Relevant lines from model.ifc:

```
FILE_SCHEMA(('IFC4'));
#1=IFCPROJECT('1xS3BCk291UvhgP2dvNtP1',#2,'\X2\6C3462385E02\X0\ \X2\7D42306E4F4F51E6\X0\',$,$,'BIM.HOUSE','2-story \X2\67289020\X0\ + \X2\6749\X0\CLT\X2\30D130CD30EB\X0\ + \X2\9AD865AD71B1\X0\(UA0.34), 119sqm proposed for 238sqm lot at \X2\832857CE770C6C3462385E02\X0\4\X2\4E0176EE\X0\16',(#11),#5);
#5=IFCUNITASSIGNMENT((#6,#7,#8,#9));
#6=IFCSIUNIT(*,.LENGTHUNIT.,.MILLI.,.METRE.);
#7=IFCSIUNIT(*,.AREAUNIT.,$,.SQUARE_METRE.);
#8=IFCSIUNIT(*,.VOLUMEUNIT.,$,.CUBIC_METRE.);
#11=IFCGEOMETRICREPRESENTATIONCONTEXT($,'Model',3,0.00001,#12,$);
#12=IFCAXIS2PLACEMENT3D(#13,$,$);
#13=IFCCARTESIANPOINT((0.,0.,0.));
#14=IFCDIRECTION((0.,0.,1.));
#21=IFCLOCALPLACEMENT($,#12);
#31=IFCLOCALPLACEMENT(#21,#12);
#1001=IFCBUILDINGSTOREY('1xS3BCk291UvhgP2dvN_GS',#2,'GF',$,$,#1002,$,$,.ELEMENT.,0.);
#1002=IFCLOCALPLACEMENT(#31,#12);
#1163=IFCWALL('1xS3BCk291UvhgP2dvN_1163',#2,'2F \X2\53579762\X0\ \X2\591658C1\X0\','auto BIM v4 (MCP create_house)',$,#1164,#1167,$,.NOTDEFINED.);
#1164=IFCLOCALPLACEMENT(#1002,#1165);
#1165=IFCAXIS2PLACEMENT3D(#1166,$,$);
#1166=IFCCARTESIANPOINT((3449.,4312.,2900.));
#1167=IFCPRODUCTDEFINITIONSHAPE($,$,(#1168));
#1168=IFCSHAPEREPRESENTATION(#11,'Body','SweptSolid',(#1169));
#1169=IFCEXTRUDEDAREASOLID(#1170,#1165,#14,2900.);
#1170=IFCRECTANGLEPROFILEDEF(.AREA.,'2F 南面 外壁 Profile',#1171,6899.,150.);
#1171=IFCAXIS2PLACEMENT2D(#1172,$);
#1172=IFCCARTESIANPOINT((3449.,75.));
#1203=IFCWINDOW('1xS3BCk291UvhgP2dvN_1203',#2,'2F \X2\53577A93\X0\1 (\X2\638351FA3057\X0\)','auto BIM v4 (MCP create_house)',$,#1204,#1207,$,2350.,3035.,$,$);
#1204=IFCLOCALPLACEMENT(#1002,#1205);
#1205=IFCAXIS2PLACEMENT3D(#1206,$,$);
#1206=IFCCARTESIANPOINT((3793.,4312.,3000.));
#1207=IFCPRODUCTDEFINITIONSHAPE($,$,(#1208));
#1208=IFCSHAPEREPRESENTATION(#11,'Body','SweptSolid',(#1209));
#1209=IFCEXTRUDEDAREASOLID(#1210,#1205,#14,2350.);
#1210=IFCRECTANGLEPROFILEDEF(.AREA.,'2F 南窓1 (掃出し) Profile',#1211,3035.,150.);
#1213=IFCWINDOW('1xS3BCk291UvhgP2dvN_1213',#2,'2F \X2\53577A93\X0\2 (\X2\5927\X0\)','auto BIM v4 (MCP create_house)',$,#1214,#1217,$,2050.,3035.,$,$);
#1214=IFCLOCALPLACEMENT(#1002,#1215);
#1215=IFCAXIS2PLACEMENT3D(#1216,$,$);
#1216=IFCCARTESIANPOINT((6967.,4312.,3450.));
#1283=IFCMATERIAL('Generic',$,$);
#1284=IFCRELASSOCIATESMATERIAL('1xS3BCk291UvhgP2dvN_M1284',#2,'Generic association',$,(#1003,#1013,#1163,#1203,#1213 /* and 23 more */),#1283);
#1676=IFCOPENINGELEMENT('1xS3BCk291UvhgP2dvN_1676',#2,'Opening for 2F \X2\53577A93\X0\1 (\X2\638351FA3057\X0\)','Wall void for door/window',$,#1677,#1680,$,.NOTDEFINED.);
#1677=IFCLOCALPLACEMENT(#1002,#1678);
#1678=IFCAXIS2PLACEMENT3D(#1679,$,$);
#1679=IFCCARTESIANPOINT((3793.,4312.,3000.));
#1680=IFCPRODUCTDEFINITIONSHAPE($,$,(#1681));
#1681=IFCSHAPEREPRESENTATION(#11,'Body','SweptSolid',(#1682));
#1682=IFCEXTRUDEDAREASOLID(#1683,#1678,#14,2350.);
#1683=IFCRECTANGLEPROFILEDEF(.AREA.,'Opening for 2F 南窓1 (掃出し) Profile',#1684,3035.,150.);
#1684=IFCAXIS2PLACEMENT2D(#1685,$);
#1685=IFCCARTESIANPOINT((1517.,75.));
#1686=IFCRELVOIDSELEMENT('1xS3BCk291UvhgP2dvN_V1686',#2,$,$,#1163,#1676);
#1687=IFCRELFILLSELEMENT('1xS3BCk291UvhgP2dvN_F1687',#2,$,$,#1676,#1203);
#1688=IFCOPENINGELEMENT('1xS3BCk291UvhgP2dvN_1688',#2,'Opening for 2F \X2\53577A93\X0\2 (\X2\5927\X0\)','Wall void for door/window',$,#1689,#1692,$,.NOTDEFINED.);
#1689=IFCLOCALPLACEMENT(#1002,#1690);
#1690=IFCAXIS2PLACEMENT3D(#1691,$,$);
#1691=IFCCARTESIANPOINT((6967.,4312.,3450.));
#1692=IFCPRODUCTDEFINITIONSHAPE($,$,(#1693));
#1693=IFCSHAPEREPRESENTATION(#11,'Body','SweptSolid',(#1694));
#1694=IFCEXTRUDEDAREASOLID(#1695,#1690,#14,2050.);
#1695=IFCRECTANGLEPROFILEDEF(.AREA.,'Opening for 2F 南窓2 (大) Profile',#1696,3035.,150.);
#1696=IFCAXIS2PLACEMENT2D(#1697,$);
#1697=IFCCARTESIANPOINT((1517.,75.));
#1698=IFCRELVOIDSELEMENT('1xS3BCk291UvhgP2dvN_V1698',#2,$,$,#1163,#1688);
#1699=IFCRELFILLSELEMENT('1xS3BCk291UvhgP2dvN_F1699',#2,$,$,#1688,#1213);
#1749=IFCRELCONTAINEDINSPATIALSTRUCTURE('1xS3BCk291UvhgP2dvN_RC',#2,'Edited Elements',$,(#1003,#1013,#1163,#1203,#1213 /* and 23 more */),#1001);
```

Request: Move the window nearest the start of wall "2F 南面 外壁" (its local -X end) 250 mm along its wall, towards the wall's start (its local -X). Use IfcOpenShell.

```python
import ifcopenshell
import ifcopenshell.api.geometry
import ifcopenshell.util.placement

model = ifcopenshell.open("model.ifc")

window = model.by_id(1203)
opening = window.FillsVoids[0].RelatingOpeningElement
wall = opening.VoidsElements[0].RelatingBuildingElement

wall_matrix = ifcopenshell.util.placement.get_local_placement(wall.ObjectPlacement)
shift = wall_matrix[:3, 0] * -250.0
before = ifcopenshell.util.placement.get_local_placement(window.ObjectPlacement)[:3, 3].copy()

# The window is not placed relative to its opening, so move both.
for product in (opening, window):
    matrix = ifcopenshell.util.placement.get_local_placement(product.ObjectPlacement)
    matrix[:3, 3] += shift
    ifcopenshell.api.geometry.edit_object_placement(model, product=product, matrix=matrix, is_si=False)

after = ifcopenshell.util.placement.get_local_placement(window.ObjectPlacement)[:3, 3]
print("window moved by", (after - before).round(3) + 0.0)

model.write("model_rev.ifc")
```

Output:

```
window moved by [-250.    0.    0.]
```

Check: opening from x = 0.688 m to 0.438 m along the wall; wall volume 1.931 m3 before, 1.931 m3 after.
